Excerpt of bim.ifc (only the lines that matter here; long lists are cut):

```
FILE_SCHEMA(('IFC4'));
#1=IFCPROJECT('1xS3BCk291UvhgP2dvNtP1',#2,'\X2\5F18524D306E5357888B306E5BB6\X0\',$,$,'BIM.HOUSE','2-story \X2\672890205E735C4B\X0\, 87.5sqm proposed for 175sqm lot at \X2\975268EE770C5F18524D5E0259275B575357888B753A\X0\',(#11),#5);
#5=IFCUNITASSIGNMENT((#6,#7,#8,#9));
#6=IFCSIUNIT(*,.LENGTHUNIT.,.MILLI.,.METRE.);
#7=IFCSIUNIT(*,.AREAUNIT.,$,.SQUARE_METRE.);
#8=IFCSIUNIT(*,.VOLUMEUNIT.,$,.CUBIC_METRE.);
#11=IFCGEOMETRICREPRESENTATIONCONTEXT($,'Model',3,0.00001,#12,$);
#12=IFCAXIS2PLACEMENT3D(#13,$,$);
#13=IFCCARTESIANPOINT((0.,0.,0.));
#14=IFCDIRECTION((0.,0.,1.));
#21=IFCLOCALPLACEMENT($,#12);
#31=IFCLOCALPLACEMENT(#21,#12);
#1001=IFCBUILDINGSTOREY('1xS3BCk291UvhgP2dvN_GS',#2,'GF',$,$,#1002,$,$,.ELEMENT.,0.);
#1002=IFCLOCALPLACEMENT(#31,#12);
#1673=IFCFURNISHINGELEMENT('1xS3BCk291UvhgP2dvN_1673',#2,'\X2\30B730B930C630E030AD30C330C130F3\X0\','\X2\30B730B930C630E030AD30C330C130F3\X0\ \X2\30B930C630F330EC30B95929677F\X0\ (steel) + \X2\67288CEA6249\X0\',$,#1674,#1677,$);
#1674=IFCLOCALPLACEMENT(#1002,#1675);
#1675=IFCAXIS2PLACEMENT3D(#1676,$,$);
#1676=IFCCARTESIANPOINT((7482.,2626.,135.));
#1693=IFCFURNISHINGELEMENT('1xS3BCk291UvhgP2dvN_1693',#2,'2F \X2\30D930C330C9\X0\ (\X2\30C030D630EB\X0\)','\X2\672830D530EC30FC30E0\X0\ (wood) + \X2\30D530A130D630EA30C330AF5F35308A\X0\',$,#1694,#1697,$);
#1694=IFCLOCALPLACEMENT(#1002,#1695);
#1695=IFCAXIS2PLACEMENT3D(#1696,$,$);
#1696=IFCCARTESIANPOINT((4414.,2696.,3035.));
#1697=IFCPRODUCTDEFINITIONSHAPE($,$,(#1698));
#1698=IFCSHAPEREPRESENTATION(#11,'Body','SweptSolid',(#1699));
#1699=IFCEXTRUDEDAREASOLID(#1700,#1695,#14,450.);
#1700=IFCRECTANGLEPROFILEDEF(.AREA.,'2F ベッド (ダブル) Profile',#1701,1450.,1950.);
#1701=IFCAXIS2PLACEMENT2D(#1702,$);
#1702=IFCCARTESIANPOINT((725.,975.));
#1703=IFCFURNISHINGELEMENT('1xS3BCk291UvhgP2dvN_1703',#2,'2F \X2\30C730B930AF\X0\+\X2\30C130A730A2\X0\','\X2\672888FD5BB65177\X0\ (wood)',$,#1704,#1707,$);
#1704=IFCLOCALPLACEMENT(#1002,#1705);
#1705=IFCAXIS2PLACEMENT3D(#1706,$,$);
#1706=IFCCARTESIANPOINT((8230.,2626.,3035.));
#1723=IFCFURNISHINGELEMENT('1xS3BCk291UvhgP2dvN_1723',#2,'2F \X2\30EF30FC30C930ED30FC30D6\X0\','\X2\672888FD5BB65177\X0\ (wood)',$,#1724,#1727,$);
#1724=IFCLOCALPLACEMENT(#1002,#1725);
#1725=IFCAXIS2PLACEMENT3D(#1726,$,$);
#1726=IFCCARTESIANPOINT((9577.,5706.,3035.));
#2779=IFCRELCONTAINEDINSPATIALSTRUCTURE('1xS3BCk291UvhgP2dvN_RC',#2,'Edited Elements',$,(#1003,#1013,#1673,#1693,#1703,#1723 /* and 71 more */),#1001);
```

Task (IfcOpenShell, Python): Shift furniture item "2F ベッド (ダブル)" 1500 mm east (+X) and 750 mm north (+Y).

```python
import ifcopenshell
import ifcopenshell.api.geometry
import ifcopenshell.util.placement
import ifcopenshell.util.unit

model = ifcopenshell.open("bim.ifc")
unit_scale = ifcopenshell.util.unit.calculate_unit_scale(model)

item = model.by_guid("1xS3BCk291UvhgP2dvN_1693")
matrix = ifcopenshell.util.placement.get_local_placement(item.ObjectPlacement)
matrix[0, 3] += 1.5 / unit_scale
matrix[1, 3] += 0.75 / unit_scale
ifcopenshell.api.geometry.edit_object_placement(model, product=item, matrix=matrix, is_si=False)

print(ifcopenshell.util.placement.get_local_placement(item.ObjectPlacement).round(3) + 0.0)

model.write("bim_rev.ifc")
```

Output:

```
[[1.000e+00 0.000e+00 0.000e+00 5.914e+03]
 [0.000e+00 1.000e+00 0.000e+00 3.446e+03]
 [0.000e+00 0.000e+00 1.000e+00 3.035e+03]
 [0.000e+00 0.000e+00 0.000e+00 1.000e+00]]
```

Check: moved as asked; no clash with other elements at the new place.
